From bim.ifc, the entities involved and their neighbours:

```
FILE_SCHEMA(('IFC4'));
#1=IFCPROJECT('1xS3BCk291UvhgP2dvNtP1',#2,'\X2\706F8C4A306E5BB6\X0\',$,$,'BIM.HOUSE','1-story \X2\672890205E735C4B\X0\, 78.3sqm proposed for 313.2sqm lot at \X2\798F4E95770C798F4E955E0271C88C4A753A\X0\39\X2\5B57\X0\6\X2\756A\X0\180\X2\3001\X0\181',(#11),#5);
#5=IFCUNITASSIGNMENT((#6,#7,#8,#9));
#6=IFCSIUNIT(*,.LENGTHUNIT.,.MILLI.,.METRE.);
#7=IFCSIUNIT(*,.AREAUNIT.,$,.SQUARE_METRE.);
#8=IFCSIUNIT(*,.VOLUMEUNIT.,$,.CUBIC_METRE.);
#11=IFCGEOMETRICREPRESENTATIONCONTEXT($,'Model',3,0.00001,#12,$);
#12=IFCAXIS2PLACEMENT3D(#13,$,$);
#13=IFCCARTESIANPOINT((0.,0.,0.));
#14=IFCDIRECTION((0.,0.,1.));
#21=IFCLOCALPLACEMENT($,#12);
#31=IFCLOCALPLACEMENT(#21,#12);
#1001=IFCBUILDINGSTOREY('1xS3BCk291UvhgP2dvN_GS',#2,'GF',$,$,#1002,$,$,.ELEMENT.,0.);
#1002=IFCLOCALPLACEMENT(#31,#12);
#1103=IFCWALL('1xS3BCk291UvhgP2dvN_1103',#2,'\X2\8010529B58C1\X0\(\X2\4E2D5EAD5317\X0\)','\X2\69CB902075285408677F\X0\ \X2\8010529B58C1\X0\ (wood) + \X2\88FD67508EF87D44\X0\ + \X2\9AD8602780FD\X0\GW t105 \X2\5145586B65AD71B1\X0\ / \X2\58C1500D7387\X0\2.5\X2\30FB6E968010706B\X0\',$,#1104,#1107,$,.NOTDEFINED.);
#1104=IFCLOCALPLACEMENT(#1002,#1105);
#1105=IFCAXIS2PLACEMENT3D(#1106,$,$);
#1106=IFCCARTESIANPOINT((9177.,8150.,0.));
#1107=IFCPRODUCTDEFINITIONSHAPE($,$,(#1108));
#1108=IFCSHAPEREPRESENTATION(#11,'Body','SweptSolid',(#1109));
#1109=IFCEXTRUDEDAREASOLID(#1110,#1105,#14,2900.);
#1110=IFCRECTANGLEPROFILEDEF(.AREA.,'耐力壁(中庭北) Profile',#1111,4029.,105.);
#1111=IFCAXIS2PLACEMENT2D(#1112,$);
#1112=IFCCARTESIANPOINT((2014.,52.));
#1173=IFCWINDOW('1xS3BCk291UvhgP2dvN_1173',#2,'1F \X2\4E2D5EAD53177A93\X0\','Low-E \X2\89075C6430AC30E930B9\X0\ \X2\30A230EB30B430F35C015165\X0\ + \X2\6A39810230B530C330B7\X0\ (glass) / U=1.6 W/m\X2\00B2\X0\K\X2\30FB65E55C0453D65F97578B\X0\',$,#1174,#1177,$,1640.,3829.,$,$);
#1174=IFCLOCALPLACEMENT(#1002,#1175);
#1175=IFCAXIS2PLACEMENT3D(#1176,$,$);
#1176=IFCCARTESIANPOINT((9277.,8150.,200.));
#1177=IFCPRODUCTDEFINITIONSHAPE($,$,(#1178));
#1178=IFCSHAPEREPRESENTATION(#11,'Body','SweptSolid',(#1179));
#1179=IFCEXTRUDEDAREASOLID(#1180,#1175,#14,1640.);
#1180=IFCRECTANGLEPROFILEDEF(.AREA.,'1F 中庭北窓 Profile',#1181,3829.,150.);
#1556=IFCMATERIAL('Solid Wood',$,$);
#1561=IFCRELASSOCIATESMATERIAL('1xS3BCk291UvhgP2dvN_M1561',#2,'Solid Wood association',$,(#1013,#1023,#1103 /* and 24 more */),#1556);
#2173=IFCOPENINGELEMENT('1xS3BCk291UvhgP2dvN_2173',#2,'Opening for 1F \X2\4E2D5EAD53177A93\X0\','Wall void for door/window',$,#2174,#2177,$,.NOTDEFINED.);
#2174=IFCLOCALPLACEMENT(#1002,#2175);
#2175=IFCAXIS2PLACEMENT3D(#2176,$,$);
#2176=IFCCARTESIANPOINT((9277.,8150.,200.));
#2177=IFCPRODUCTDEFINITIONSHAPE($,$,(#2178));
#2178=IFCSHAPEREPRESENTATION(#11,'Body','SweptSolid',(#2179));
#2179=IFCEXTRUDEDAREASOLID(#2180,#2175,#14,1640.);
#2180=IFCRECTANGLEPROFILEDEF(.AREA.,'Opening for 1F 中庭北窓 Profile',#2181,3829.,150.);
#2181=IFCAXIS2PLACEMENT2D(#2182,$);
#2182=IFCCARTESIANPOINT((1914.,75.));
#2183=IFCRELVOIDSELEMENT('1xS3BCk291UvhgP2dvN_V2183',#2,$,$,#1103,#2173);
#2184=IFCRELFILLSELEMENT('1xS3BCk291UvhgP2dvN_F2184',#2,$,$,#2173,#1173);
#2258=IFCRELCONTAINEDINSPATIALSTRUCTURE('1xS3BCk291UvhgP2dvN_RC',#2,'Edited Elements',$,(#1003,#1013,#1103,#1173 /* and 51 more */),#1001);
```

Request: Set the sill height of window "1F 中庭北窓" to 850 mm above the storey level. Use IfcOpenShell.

```python
import numpy as np
import ifcopenshell
import ifcopenshell.api.geometry
import ifcopenshell.geom
import ifcopenshell.util.element
import ifcopenshell.util.placement
import ifcopenshell.util.shape
import ifcopenshell.util.unit

model = ifcopenshell.open("bim.ifc")
unit_scale = ifcopenshell.util.unit.calculate_unit_scale(model)

window = model.by_id(1173)
opening = window.FillsVoids[0].RelatingOpeningElement
storey = ifcopenshell.util.element.get_container(window, ifc_class="IfcBuildingStorey")
level = ifcopenshell.util.placement.get_local_placement(storey.ObjectPlacement)[2, 3]

# The opening's origin need not be at the sill, so measure its lowest point.
shape = ifcopenshell.geom.create_shape(ifcopenshell.geom.settings(), opening)
bottom = ifcopenshell.util.shape.get_shape_bottom_elevation(shape, shape.geometry) / unit_scale
dz = level + 0.85 / unit_scale - bottom

shift = np.array([0.0, 0.0, dz])
# The window is not placed relative to its opening, so move both.
for product in (opening, window):
    matrix = ifcopenshell.util.placement.get_local_placement(product.ObjectPlacement)
    matrix[:3, 3] += shift
    ifcopenshell.api.geometry.edit_object_placement(model, product=product, matrix=matrix, is_si=False)

print(f"moved by {dz * unit_scale:+.3f} m")

model.write("bim_v2.ifc")
```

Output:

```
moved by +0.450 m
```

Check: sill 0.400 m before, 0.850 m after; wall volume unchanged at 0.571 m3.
